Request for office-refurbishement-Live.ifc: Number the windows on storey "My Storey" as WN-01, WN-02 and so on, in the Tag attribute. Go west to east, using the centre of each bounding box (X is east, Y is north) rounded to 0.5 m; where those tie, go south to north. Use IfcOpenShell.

First a look at what the model holds.

```python
import ifcopenshell
import ifcopenshell.util.element
import ifcopenshell.util.placement

model = ifcopenshell.open("office-refurbishement-Live.ifc")
print(model.schema)
storey = next(s for s in model.by_type("IfcBuildingStorey") if s.Name == "My Storey")
windows = [e for e in ifcopenshell.util.element.get_decomposition(storey) if e.is_a("IfcWindow")]
for e in sorted(windows, key=lambda e: e.id()):
    origin = ifcopenshell.util.placement.get_local_placement(e.ObjectPlacement)[:3, 3]
    print(e.id(), e.Tag, e.Name, origin.round(2) + 0.0, sep=" | ")
```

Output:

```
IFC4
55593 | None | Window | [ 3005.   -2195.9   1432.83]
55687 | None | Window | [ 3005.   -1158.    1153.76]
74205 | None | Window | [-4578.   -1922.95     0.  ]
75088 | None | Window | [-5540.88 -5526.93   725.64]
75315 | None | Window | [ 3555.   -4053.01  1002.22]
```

```python
import ifcopenshell
import ifcopenshell.geom
import ifcopenshell.util.element
import ifcopenshell.util.shape

model = ifcopenshell.open("office-refurbishement-Live.ifc")
settings = ifcopenshell.geom.settings()
settings.set("use-world-coords", True)


def centre(element):
    shape = ifcopenshell.geom.create_shape(settings, element)
    return ifcopenshell.util.shape.get_bbox_centroid(shape.geometry)


storey = next(s for s in model.by_type("IfcBuildingStorey") if s.Name == "My Storey")
windows = [e for e in ifcopenshell.util.element.get_decomposition(storey) if e.is_a("IfcWindow")]

# Insertion points can sit at a corner or the storey origin, so sort by the geometry (in metres).
centres = {e: centre(e) for e in windows}
windows.sort(key=lambda e: (round(centres[e][0] / 0.5), centres[e][1]))

for i, e in enumerate(windows, start=1):
    number = f"WN-{i:02d}"
    e.Tag = number
    print(e.id(), number)

model.write("office-refurbishement-Live_rev.ifc")
```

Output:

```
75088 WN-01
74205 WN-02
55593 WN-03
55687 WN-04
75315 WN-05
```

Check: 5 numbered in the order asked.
